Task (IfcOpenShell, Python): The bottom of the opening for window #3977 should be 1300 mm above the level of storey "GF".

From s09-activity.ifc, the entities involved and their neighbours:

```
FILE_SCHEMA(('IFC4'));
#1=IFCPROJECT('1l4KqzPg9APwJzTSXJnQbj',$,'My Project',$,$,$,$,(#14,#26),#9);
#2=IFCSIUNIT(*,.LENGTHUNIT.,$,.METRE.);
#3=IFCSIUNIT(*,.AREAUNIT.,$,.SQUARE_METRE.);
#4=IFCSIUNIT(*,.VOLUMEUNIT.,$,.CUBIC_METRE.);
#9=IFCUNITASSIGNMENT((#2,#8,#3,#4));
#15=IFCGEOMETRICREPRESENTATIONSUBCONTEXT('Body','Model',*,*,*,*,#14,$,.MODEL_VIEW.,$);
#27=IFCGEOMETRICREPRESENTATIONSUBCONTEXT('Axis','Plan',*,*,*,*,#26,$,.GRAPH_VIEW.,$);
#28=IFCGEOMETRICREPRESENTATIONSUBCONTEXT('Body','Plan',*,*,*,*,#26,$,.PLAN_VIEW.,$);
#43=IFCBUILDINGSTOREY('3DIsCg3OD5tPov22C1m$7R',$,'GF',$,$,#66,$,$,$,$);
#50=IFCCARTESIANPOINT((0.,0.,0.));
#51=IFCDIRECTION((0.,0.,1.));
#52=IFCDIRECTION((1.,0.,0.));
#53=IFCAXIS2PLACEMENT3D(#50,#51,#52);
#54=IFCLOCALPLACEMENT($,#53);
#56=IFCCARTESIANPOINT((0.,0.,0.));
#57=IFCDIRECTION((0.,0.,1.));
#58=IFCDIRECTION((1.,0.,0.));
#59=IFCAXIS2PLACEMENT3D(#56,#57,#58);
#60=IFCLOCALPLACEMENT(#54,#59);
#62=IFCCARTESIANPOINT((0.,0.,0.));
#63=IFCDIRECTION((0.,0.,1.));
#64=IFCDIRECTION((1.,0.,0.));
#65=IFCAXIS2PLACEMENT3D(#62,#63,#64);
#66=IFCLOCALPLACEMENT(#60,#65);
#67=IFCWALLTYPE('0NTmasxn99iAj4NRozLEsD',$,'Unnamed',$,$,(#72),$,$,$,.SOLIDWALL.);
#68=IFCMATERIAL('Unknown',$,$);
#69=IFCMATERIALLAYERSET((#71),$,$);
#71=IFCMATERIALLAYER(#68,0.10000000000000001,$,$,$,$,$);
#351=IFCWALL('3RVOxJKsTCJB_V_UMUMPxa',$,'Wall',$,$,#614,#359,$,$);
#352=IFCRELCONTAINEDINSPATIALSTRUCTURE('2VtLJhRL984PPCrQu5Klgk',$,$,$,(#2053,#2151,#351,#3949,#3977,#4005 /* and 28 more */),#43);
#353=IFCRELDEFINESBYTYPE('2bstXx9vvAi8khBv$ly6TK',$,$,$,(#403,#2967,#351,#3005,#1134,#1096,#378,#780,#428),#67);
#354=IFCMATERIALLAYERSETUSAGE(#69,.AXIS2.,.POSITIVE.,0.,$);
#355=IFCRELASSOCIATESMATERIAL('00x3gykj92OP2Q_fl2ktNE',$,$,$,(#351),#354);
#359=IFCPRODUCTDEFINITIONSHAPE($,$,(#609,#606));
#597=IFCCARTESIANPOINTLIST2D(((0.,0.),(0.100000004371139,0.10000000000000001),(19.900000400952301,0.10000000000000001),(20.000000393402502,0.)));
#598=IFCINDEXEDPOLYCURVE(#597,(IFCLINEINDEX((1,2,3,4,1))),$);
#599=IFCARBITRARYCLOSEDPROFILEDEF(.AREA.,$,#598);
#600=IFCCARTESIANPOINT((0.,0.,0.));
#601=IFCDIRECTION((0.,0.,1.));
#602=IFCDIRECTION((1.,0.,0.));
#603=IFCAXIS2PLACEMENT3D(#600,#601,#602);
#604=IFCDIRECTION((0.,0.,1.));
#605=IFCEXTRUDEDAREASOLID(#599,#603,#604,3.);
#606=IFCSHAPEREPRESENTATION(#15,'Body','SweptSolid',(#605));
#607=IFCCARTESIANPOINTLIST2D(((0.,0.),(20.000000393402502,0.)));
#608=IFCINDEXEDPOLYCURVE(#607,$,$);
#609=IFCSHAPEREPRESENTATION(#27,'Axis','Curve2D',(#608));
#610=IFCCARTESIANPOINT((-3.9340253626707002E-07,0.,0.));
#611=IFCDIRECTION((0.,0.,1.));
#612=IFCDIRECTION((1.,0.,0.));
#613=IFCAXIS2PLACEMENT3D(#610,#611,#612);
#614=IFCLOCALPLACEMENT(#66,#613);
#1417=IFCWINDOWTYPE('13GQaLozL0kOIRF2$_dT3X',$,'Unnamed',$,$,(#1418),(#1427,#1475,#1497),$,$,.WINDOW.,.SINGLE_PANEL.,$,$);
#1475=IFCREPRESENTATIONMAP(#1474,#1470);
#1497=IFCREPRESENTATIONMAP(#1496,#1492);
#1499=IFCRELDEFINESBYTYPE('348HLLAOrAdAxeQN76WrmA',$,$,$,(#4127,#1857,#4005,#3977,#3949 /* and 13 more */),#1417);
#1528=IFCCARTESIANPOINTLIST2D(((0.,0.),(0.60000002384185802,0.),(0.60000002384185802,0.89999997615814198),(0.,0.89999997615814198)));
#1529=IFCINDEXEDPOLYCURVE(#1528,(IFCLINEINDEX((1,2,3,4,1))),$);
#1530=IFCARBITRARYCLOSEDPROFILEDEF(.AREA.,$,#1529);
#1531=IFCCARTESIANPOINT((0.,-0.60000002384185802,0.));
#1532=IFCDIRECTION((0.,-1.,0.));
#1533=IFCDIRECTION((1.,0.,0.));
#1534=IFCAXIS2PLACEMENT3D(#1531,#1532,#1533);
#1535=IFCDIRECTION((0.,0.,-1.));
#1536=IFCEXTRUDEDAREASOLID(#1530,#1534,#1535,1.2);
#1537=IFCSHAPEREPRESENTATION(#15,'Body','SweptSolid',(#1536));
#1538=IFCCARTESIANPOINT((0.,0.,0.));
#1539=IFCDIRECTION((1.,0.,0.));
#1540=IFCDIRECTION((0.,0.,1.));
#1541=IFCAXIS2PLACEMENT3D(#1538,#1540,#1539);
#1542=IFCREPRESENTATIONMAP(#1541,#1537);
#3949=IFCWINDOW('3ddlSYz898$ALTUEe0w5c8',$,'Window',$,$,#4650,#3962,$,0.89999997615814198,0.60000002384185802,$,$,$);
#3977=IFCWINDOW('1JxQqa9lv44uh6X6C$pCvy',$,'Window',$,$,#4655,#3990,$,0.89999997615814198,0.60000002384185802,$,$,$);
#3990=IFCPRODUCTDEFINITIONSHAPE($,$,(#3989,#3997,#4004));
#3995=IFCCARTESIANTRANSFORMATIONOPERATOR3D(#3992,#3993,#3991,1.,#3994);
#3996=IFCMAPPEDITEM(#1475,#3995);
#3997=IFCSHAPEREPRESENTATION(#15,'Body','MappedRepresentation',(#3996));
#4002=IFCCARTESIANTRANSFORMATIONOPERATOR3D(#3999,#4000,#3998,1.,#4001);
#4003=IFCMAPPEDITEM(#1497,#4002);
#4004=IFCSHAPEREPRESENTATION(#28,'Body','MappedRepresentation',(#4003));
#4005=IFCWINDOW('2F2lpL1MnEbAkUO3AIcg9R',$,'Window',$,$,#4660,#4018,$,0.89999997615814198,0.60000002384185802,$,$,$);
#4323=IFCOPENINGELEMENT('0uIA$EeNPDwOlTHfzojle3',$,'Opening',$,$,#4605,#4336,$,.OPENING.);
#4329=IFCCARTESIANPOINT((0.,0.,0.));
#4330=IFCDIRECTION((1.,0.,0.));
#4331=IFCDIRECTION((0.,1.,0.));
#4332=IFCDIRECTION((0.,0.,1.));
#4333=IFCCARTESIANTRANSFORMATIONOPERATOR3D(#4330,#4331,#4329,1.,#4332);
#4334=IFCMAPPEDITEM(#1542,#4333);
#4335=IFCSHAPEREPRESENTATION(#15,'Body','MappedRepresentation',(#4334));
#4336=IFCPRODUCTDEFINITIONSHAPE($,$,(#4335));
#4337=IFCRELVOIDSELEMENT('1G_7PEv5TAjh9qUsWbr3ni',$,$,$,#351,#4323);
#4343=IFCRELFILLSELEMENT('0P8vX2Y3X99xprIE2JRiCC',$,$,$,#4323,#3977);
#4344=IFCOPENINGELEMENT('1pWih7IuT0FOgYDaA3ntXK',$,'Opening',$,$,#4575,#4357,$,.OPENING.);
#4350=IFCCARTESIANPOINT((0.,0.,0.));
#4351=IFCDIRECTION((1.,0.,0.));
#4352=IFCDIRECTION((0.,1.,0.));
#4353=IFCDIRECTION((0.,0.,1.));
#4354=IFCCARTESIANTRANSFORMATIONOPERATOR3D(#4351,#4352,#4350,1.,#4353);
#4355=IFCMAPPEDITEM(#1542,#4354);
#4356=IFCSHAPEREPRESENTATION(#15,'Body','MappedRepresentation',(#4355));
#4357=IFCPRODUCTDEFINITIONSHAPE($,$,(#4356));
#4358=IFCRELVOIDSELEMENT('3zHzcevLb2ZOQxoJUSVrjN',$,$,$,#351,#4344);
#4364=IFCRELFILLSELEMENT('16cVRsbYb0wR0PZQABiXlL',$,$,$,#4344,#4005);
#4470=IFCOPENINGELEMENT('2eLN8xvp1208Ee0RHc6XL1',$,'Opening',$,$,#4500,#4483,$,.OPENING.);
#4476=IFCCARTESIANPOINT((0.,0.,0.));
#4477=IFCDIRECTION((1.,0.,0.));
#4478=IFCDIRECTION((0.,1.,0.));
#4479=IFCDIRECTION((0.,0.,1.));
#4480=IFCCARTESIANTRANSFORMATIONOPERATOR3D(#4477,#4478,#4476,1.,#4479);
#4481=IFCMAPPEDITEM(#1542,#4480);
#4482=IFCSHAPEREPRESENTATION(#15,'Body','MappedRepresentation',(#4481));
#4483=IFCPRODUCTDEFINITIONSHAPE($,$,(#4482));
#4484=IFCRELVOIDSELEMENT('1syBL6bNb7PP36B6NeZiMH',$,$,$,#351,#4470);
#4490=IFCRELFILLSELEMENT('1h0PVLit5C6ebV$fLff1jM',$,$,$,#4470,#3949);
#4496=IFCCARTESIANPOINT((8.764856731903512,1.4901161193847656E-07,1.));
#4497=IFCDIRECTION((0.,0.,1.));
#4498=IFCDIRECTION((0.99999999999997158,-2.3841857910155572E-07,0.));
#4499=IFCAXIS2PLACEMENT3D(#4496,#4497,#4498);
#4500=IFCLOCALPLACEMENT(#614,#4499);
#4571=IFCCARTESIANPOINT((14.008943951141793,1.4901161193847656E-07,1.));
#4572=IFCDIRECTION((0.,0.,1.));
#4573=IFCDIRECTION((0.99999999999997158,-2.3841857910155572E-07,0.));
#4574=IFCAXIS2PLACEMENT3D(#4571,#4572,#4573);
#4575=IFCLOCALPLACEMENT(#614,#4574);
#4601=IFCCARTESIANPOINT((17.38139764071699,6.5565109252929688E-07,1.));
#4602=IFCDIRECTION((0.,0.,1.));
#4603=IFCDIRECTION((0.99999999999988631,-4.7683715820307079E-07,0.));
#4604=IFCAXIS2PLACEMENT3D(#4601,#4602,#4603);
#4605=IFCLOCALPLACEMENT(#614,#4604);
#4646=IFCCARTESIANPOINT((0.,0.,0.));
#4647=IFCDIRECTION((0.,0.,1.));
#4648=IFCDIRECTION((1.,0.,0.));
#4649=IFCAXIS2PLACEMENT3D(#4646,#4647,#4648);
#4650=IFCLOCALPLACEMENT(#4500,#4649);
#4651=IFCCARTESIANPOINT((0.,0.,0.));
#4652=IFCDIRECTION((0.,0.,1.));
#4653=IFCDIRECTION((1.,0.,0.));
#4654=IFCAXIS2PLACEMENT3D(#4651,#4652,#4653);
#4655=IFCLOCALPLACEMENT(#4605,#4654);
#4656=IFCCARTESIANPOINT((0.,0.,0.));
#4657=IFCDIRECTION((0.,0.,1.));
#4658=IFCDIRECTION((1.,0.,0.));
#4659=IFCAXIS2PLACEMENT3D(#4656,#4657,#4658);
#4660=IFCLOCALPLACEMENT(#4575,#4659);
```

```python
import numpy as np
import ifcopenshell
import ifcopenshell.api.geometry
import ifcopenshell.geom
import ifcopenshell.util.element
import ifcopenshell.util.placement
import ifcopenshell.util.shape
import ifcopenshell.util.unit

model = ifcopenshell.open("s09-activity.ifc")
unit_scale = ifcopenshell.util.unit.calculate_unit_scale(model)

window = model.by_guid("1JxQqa9lv44uh6X6C$pCvy")
opening = window.FillsVoids[0].RelatingOpeningElement
storey = ifcopenshell.util.element.get_container(window, ifc_class="IfcBuildingStorey")
level = ifcopenshell.util.placement.get_local_placement(storey.ObjectPlacement)[2, 3]

# The opening's origin need not be at the sill, so measure its lowest point.
shape = ifcopenshell.geom.create_shape(ifcopenshell.geom.settings(), opening)
bottom = ifcopenshell.util.shape.get_shape_bottom_elevation(shape, shape.geometry) / unit_scale
dz = level + 1.3 / unit_scale - bottom

shift = np.array([0.0, 0.0, dz])
# The window is placed relative to its opening, so it follows when the opening moves.
matrix = ifcopenshell.util.placement.get_local_placement(opening.ObjectPlacement)
matrix[:3, 3] += shift
ifcopenshell.api.geometry.edit_object_placement(
    model, product=opening, matrix=matrix, is_si=False, should_transform_children=True
)

print(f"moved by {dz * unit_scale:+.3f} m")

model.write("s09-activity_edited.ifc")
```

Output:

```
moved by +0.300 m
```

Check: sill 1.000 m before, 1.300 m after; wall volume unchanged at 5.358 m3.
